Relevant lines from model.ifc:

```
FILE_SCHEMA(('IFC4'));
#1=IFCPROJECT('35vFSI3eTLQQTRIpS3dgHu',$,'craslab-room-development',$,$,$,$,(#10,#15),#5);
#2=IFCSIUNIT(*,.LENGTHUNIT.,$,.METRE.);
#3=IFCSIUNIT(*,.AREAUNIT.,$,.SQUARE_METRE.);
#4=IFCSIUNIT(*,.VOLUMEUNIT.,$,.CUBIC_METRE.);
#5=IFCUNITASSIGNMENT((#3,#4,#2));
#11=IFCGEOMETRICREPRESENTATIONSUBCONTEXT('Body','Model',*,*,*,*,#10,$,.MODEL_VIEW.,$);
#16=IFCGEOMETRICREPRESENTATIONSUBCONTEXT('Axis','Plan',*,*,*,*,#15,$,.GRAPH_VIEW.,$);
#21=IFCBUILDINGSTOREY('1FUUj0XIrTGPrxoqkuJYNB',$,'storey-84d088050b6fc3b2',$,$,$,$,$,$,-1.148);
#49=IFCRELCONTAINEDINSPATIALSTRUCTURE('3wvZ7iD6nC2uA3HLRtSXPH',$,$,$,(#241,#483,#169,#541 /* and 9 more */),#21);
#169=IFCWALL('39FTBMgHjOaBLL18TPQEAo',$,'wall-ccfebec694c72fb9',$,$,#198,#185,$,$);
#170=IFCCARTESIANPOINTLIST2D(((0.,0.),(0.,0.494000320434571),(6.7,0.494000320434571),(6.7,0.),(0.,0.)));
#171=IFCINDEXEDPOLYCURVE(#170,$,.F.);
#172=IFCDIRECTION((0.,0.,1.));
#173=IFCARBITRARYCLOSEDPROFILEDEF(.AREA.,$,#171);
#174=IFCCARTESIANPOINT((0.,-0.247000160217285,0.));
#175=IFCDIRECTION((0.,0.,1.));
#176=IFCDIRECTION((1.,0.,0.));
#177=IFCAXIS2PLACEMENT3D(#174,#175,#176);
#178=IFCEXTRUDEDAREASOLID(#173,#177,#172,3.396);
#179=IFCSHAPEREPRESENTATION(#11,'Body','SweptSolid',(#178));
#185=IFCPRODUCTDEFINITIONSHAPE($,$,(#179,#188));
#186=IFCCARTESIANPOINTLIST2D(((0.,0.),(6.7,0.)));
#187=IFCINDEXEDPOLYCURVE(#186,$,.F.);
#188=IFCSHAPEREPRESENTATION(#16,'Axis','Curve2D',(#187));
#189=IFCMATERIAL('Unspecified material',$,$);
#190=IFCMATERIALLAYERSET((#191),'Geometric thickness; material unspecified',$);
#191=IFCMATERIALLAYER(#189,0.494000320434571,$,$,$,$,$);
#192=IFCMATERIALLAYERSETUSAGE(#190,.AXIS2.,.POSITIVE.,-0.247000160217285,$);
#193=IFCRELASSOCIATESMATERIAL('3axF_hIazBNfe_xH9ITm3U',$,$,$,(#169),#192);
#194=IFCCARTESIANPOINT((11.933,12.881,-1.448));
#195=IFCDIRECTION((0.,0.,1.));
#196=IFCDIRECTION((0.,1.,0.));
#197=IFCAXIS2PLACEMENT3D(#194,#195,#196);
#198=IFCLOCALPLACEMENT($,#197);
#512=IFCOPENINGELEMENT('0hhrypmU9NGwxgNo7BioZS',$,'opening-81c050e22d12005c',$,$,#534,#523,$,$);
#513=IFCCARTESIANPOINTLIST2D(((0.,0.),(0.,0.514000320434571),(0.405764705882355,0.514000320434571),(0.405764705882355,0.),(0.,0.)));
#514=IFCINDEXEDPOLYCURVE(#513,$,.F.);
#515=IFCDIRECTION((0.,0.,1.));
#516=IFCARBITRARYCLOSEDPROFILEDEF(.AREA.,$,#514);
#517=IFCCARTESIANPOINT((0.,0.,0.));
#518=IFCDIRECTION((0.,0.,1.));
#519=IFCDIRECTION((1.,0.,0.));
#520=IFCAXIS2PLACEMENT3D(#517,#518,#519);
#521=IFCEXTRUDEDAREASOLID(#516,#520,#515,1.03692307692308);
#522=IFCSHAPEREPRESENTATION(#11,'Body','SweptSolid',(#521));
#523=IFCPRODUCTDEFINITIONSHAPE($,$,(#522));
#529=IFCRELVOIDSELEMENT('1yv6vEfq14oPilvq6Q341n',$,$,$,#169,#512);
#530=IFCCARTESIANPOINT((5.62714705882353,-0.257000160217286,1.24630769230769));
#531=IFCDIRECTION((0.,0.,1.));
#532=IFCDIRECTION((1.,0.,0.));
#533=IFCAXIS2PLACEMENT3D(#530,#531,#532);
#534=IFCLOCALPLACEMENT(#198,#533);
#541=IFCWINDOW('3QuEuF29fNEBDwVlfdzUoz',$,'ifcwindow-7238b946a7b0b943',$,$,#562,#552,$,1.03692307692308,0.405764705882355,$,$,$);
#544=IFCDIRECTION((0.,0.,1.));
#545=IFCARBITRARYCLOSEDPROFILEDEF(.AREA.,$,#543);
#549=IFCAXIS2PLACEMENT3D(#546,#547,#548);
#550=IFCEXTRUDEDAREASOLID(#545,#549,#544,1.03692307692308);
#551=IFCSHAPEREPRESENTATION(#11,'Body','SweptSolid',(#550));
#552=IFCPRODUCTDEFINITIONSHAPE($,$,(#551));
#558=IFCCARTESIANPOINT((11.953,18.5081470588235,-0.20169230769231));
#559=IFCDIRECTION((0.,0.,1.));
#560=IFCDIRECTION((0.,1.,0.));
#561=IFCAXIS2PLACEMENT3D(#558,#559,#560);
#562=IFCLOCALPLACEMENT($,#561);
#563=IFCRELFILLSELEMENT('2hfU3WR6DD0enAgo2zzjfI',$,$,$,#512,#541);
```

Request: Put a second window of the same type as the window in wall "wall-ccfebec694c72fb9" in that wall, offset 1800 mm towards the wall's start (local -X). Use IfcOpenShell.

```python
import ifcopenshell
import ifcopenshell.api.feature
import ifcopenshell.api.geometry
import ifcopenshell.api.root
import ifcopenshell.geom
import ifcopenshell.util.element
import ifcopenshell.util.placement
import ifcopenshell.util.shape

model = ifcopenshell.open("model.ifc")
settings = ifcopenshell.geom.settings()


def volume(element):
    """Net volume in cubic metres, openings subtracted."""
    shape = ifcopenshell.geom.create_shape(settings, element)
    return ifcopenshell.util.shape.get_volume(shape.geometry)


window = model.by_guid("3QuEuF29fNEBDwVlfdzUoz")
opening = window.FillsVoids[0].RelatingOpeningElement
wall = opening.VoidsElements[0].RelatingBuildingElement
before = volume(wall)
shift = ifcopenshell.util.placement.get_local_placement(wall.ObjectPlacement)[:3, 0] * -1.8

# copy_class copies the void relationship, type, container and properties, but no geometry.
new_opening = ifcopenshell.api.root.copy_class(model, product=opening)
new_opening.Representation = ifcopenshell.util.element.copy_deep(
    model, opening.Representation, exclude=["IfcGeometricRepresentationContext", "IfcRepresentationMap"]
)
new_window = ifcopenshell.api.root.copy_class(model, product=window)
new_window.Representation = ifcopenshell.util.element.copy_deep(
    model, window.Representation, exclude=["IfcGeometricRepresentationContext", "IfcRepresentationMap"]
)
ifcopenshell.api.feature.add_filling(model, opening=new_opening, element=new_window)

for old, new in ((opening, new_opening), (window, new_window)):
    matrix = ifcopenshell.util.placement.get_local_placement(old.ObjectPlacement)
    matrix[:3, 3] += shift
    ifcopenshell.api.geometry.edit_object_placement(model, product=new, matrix=matrix, is_si=False)

after = volume(wall)

print(f"wall volume {before:.3f} -> {after:.3f} m3")

model.write("model-out.ifc")
```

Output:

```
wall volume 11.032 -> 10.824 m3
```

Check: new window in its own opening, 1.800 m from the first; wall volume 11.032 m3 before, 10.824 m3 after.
